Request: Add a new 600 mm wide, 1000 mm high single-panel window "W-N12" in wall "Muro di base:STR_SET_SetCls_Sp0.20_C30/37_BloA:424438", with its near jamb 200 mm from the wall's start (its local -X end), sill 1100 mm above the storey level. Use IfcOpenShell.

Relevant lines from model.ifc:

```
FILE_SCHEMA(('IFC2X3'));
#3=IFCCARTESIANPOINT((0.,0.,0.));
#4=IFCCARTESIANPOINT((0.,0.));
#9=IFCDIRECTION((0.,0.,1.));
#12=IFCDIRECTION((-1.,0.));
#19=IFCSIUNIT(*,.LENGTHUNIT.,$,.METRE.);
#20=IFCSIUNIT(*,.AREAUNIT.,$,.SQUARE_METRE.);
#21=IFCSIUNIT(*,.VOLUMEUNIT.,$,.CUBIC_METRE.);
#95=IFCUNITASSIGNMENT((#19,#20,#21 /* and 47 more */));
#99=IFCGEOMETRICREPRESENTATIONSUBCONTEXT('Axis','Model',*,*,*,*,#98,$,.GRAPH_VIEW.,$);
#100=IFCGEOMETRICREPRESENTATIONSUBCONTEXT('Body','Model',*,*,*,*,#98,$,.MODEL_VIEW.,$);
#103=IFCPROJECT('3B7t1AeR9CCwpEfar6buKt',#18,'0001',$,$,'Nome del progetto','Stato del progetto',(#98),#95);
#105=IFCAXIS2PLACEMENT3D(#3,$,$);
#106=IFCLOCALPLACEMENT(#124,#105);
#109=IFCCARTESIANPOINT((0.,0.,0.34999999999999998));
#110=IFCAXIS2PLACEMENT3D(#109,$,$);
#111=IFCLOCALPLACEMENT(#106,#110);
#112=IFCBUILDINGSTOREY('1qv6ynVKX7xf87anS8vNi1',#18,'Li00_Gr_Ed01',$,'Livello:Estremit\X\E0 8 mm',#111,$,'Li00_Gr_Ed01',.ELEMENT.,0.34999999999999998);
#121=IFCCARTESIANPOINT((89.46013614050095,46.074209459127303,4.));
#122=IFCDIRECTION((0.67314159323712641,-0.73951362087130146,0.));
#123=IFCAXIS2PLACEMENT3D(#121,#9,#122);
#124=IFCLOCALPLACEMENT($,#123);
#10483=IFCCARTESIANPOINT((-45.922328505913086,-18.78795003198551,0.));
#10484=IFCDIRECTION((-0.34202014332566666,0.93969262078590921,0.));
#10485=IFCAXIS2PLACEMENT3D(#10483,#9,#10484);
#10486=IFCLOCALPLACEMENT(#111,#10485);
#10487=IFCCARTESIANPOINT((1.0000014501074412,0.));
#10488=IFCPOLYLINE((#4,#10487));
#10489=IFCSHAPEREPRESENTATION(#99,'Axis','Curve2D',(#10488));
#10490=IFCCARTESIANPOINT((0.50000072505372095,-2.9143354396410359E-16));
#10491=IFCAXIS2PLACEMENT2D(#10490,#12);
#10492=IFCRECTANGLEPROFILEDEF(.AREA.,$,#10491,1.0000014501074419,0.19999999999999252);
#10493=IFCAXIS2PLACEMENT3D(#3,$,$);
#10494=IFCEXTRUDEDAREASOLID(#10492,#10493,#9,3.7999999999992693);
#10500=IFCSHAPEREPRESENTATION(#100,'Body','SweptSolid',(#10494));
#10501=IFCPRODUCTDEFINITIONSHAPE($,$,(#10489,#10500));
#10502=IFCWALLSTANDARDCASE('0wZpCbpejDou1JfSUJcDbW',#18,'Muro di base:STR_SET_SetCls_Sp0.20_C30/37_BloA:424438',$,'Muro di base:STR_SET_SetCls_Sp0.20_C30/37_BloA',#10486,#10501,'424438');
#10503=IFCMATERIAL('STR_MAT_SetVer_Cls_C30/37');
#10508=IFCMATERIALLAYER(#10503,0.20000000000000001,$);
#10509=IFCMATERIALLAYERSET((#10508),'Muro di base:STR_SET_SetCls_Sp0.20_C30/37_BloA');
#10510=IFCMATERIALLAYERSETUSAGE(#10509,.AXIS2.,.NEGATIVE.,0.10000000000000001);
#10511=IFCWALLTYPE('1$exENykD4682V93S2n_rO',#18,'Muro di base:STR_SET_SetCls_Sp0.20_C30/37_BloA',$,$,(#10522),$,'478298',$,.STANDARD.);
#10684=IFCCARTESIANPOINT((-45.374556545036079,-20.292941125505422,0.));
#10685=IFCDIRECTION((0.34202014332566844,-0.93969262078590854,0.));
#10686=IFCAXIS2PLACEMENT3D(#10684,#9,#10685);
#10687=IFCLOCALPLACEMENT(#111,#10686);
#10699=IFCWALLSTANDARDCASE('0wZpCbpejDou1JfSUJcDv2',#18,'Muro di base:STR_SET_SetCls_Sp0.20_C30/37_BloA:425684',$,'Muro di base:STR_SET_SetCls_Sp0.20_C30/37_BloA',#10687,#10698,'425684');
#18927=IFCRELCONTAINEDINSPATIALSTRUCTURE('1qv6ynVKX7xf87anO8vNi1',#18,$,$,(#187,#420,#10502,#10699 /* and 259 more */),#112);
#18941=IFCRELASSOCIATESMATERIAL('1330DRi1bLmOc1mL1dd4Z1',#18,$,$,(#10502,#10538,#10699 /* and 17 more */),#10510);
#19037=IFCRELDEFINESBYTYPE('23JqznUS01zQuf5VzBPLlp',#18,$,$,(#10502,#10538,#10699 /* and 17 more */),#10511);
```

```python
import numpy as np
import ifcopenshell
import ifcopenshell.api.feature
import ifcopenshell.api.geometry
import ifcopenshell.api.root
import ifcopenshell.api.spatial
import ifcopenshell.api.type
import ifcopenshell.geom
import ifcopenshell.util.element
import ifcopenshell.util.placement
import ifcopenshell.util.representation
import ifcopenshell.util.shape
import ifcopenshell.util.unit

model = ifcopenshell.open("model.ifc")
unit_scale = ifcopenshell.util.unit.calculate_unit_scale(model)
settings = ifcopenshell.geom.settings()


def volume(element):
    """Net volume in cubic metres, openings subtracted."""
    shape = ifcopenshell.geom.create_shape(settings, element)
    return ifcopenshell.util.shape.get_volume(shape.geometry)


wall = model.by_id(10502)
storey = ifcopenshell.util.element.get_container(wall, ifc_class="IfcBuildingStorey")
context = ifcopenshell.util.representation.get_context(model, "Model", "Body", "MODEL_VIEW")
before = volume(wall)

width, height, from_end, sill = 0.6, 1, 0.2, 1.1  # metres

# The wall runs along its own X axis, and the end named is its -X end.
wall_shape = ifcopenshell.geom.create_shape(settings, wall)
x, y, z = ifcopenshell.util.shape.get_vertices(wall_shape.geometry).T
start = x.min() + from_end
face, thickness = float(y.min()), float(y.max() - y.min())
wall_matrix = ifcopenshell.util.placement.get_local_placement(wall.ObjectPlacement)
level = ifcopenshell.util.placement.get_local_placement(storey.ObjectPlacement)[2, 3]


def in_wall(x, y):
    """Placement at x, y metres in the wall's axes, at sill height."""
    matrix = wall_matrix.copy()
    matrix[:, 3] = wall_matrix @ np.array([x / unit_scale, y / unit_scale, 0.0, 1.0])
    matrix[2, 3] = level + sill / unit_scale
    return matrix


# Opening: a box that overshoots both wall faces by 50 mm.
opening = ifcopenshell.api.root.create_entity(model, ifc_class="IfcOpeningElement")
box = ifcopenshell.api.geometry.add_wall_representation(
    model, context=context, length=width, height=height, thickness=thickness + 0.1
)
ifcopenshell.api.geometry.assign_representation(model, product=opening, representation=box)
ifcopenshell.api.geometry.edit_object_placement(model, product=opening, matrix=in_wall(start, face - 0.05), is_si=False)
ifcopenshell.api.feature.add_feature(model, feature=opening, element=wall)

window = ifcopenshell.api.root.create_entity(model, ifc_class="IfcWindow", name="W-N12")
window.OverallWidth, window.OverallHeight = width / unit_scale, height / unit_scale
body = ifcopenshell.api.geometry.add_window_representation(
    model,
    context=context,
    overall_width=window.OverallWidth,
    overall_height=window.OverallHeight,
    partition_type="SINGLE_PANEL",
)
ifcopenshell.api.geometry.assign_representation(model, product=window, representation=body)
ifcopenshell.api.spatial.assign_container(model, products=[window], relating_structure=storey)
fills = ifcopenshell.api.feature.add_filling(model, opening=opening, element=window)
fills.OwnerHistory = window.OwnerHistory  # required in IFC2X3

# IFC2X3 keeps the operation on the window style.
style = ifcopenshell.api.root.create_entity(model, ifc_class="IfcWindowStyle", name="W-N12")
style.OperationType, style.ConstructionType = "SINGLE_PANEL", "NOTDEFINED"
style.ParameterTakesPrecedence = style.Sizeable = False
ifcopenshell.api.type.assign_type(model, related_objects=[window], relating_type=style)

# Centre the window in the wall's thickness.
ifcopenshell.api.geometry.edit_object_placement(model, product=window, matrix=in_wall(start, face), is_si=False)
window_shape = ifcopenshell.geom.create_shape(settings, window)
depth = ifcopenshell.util.shape.get_vertices(window_shape.geometry)[:, 1]
offset = face + thickness / 2 - (depth.min() + depth.max()) / 2
ifcopenshell.api.geometry.edit_object_placement(model, product=window, matrix=in_wall(start, offset), is_si=False)

after = volume(wall)

print(f"wall volume {before:.3f} -> {after:.3f} m3")

model.write("model-out.ifc")
```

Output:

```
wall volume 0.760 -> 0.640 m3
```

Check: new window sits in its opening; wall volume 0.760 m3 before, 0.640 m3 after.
